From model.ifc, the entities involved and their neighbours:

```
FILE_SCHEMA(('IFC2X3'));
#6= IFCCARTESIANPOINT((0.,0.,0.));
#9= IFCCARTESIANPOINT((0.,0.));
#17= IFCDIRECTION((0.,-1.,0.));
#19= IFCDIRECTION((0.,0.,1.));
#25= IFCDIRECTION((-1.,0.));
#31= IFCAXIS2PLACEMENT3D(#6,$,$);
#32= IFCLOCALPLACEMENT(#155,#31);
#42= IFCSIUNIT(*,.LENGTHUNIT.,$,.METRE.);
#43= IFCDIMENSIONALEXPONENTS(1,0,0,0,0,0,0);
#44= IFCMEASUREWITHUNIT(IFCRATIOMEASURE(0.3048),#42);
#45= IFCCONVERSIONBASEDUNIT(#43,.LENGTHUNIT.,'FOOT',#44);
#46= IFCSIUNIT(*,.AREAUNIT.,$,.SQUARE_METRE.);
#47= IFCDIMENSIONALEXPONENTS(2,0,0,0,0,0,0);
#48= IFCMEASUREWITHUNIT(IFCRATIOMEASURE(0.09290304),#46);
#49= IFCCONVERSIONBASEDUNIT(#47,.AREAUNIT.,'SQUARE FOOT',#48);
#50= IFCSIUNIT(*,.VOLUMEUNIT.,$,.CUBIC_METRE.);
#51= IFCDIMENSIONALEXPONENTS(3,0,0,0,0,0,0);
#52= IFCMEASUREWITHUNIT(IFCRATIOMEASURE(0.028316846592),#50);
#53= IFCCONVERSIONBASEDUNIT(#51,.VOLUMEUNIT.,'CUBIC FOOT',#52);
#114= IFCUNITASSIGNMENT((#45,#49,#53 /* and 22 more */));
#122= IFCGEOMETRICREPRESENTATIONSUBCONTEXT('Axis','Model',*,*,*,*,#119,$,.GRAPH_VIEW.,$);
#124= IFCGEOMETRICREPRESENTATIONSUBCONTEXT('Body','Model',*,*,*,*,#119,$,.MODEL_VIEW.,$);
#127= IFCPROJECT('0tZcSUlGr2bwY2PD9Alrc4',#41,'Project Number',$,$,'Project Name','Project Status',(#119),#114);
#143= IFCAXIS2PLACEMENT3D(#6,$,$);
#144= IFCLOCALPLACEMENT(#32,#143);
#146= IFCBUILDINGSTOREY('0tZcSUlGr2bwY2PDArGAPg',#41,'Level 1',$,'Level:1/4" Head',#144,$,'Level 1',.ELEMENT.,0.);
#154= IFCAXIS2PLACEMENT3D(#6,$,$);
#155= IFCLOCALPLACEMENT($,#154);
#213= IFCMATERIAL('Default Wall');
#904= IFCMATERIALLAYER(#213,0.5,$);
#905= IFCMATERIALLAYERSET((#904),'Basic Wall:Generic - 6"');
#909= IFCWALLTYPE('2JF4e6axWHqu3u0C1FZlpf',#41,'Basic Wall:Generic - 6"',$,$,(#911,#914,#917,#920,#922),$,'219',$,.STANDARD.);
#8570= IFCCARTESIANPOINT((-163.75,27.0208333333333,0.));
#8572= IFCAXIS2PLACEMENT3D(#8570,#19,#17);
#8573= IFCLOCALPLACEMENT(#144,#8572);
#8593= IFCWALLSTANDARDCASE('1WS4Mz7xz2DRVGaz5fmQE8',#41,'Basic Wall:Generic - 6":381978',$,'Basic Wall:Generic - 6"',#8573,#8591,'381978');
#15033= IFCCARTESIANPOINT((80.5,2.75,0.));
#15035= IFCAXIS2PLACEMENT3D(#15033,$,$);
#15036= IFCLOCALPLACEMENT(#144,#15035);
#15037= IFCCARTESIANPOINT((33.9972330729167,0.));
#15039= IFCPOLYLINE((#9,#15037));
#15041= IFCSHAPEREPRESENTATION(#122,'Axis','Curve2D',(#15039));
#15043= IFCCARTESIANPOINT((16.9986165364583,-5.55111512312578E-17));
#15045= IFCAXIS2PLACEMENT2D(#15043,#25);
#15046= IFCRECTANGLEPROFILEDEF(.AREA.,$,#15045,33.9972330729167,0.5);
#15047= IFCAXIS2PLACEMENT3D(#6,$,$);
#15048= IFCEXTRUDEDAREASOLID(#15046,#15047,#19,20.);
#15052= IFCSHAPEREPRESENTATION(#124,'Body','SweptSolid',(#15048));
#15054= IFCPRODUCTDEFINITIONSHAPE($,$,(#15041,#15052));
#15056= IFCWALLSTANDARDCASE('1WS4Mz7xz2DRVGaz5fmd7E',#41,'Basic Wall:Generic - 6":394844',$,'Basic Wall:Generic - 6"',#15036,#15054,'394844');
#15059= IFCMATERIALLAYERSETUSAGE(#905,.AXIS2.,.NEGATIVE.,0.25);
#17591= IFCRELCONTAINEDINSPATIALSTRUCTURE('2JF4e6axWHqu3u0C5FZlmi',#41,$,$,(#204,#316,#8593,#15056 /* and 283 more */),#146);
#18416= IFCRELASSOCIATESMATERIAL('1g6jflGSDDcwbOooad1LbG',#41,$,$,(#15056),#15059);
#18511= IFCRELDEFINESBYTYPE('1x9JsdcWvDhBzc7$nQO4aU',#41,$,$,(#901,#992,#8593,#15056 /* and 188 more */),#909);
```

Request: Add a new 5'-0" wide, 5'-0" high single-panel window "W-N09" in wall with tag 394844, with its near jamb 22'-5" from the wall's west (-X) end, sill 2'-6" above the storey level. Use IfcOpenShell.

```python
import numpy as np
import ifcopenshell
import ifcopenshell.api.feature
import ifcopenshell.api.geometry
import ifcopenshell.api.root
import ifcopenshell.api.spatial
import ifcopenshell.api.type
import ifcopenshell.geom
import ifcopenshell.util.element
import ifcopenshell.util.placement
import ifcopenshell.util.representation
import ifcopenshell.util.shape
import ifcopenshell.util.unit

model = ifcopenshell.open("model.ifc")
unit_scale = ifcopenshell.util.unit.calculate_unit_scale(model)
settings = ifcopenshell.geom.settings()


def volume(element):
    """Net volume in cubic metres, openings subtracted."""
    shape = ifcopenshell.geom.create_shape(settings, element)
    return ifcopenshell.util.shape.get_volume(shape.geometry)


wall = model.by_guid("1WS4Mz7xz2DRVGaz5fmd7E")
storey = ifcopenshell.util.element.get_container(wall, ifc_class="IfcBuildingStorey")
context = ifcopenshell.util.representation.get_context(model, "Model", "Body", "MODEL_VIEW")
before = volume(wall)

width, height, from_end, sill = 1.524, 1.524, 6.8326, 0.762  # metres

# The wall runs along its own X axis, and the end named is its -X end.
wall_shape = ifcopenshell.geom.create_shape(settings, wall)
x, y, z = ifcopenshell.util.shape.get_vertices(wall_shape.geometry).T
start = x.min() + from_end
face, thickness = float(y.min()), float(y.max() - y.min())
wall_matrix = ifcopenshell.util.placement.get_local_placement(wall.ObjectPlacement)
level = ifcopenshell.util.placement.get_local_placement(storey.ObjectPlacement)[2, 3]


def in_wall(x, y):
    """Placement at x, y metres in the wall's axes, at sill height."""
    matrix = wall_matrix.copy()
    matrix[:, 3] = wall_matrix @ np.array([x / unit_scale, y / unit_scale, 0.0, 1.0])
    matrix[2, 3] = level + sill / unit_scale
    return matrix


# Opening: a box that overshoots both wall faces by 50 mm.
opening = ifcopenshell.api.root.create_entity(model, ifc_class="IfcOpeningElement")
box = ifcopenshell.api.geometry.add_wall_representation(
    model, context=context, length=width, height=height, thickness=thickness + 0.1
)
ifcopenshell.api.geometry.assign_representation(model, product=opening, representation=box)
ifcopenshell.api.geometry.edit_object_placement(model, product=opening, matrix=in_wall(start, face - 0.05), is_si=False)
ifcopenshell.api.feature.add_feature(model, feature=opening, element=wall)

window = ifcopenshell.api.root.create_entity(model, ifc_class="IfcWindow", name="W-N09")
window.OverallWidth, window.OverallHeight = width / unit_scale, height / unit_scale
body = ifcopenshell.api.geometry.add_window_representation(
    model,
    context=context,
    overall_width=window.OverallWidth,
    overall_height=window.OverallHeight,
    partition_type="SINGLE_PANEL",
)
ifcopenshell.api.geometry.assign_representation(model, product=window, representation=body)
ifcopenshell.api.spatial.assign_container(model, products=[window], relating_structure=storey)
fills = ifcopenshell.api.feature.add_filling(model, opening=opening, element=window)
fills.OwnerHistory = window.OwnerHistory  # required in IFC2X3

# IFC2X3 keeps the operation on the window style.
style = ifcopenshell.api.root.create_entity(model, ifc_class="IfcWindowStyle", name="W-N09")
style.OperationType, style.ConstructionType = "SINGLE_PANEL", "NOTDEFINED"
style.ParameterTakesPrecedence = style.Sizeable = False
ifcopenshell.api.type.assign_type(model, related_objects=[window], relating_type=style)

# Centre the window in the wall's thickness.
ifcopenshell.api.geometry.edit_object_placement(model, product=window, matrix=in_wall(start, face), is_si=False)
window_shape = ifcopenshell.geom.create_shape(settings, window)
depth = ifcopenshell.util.shape.get_vertices(window_shape.geometry)[:, 1]
offset = face + thickness / 2 - (depth.min() + depth.max()) / 2
ifcopenshell.api.geometry.edit_object_placement(model, product=window, matrix=in_wall(start, offset), is_si=False)

after = volume(wall)

print(f"wall volume {before:.3f} -> {after:.3f} m3")

model.write("model_edited.ifc")
```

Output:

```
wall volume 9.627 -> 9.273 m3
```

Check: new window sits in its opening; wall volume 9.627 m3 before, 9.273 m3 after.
